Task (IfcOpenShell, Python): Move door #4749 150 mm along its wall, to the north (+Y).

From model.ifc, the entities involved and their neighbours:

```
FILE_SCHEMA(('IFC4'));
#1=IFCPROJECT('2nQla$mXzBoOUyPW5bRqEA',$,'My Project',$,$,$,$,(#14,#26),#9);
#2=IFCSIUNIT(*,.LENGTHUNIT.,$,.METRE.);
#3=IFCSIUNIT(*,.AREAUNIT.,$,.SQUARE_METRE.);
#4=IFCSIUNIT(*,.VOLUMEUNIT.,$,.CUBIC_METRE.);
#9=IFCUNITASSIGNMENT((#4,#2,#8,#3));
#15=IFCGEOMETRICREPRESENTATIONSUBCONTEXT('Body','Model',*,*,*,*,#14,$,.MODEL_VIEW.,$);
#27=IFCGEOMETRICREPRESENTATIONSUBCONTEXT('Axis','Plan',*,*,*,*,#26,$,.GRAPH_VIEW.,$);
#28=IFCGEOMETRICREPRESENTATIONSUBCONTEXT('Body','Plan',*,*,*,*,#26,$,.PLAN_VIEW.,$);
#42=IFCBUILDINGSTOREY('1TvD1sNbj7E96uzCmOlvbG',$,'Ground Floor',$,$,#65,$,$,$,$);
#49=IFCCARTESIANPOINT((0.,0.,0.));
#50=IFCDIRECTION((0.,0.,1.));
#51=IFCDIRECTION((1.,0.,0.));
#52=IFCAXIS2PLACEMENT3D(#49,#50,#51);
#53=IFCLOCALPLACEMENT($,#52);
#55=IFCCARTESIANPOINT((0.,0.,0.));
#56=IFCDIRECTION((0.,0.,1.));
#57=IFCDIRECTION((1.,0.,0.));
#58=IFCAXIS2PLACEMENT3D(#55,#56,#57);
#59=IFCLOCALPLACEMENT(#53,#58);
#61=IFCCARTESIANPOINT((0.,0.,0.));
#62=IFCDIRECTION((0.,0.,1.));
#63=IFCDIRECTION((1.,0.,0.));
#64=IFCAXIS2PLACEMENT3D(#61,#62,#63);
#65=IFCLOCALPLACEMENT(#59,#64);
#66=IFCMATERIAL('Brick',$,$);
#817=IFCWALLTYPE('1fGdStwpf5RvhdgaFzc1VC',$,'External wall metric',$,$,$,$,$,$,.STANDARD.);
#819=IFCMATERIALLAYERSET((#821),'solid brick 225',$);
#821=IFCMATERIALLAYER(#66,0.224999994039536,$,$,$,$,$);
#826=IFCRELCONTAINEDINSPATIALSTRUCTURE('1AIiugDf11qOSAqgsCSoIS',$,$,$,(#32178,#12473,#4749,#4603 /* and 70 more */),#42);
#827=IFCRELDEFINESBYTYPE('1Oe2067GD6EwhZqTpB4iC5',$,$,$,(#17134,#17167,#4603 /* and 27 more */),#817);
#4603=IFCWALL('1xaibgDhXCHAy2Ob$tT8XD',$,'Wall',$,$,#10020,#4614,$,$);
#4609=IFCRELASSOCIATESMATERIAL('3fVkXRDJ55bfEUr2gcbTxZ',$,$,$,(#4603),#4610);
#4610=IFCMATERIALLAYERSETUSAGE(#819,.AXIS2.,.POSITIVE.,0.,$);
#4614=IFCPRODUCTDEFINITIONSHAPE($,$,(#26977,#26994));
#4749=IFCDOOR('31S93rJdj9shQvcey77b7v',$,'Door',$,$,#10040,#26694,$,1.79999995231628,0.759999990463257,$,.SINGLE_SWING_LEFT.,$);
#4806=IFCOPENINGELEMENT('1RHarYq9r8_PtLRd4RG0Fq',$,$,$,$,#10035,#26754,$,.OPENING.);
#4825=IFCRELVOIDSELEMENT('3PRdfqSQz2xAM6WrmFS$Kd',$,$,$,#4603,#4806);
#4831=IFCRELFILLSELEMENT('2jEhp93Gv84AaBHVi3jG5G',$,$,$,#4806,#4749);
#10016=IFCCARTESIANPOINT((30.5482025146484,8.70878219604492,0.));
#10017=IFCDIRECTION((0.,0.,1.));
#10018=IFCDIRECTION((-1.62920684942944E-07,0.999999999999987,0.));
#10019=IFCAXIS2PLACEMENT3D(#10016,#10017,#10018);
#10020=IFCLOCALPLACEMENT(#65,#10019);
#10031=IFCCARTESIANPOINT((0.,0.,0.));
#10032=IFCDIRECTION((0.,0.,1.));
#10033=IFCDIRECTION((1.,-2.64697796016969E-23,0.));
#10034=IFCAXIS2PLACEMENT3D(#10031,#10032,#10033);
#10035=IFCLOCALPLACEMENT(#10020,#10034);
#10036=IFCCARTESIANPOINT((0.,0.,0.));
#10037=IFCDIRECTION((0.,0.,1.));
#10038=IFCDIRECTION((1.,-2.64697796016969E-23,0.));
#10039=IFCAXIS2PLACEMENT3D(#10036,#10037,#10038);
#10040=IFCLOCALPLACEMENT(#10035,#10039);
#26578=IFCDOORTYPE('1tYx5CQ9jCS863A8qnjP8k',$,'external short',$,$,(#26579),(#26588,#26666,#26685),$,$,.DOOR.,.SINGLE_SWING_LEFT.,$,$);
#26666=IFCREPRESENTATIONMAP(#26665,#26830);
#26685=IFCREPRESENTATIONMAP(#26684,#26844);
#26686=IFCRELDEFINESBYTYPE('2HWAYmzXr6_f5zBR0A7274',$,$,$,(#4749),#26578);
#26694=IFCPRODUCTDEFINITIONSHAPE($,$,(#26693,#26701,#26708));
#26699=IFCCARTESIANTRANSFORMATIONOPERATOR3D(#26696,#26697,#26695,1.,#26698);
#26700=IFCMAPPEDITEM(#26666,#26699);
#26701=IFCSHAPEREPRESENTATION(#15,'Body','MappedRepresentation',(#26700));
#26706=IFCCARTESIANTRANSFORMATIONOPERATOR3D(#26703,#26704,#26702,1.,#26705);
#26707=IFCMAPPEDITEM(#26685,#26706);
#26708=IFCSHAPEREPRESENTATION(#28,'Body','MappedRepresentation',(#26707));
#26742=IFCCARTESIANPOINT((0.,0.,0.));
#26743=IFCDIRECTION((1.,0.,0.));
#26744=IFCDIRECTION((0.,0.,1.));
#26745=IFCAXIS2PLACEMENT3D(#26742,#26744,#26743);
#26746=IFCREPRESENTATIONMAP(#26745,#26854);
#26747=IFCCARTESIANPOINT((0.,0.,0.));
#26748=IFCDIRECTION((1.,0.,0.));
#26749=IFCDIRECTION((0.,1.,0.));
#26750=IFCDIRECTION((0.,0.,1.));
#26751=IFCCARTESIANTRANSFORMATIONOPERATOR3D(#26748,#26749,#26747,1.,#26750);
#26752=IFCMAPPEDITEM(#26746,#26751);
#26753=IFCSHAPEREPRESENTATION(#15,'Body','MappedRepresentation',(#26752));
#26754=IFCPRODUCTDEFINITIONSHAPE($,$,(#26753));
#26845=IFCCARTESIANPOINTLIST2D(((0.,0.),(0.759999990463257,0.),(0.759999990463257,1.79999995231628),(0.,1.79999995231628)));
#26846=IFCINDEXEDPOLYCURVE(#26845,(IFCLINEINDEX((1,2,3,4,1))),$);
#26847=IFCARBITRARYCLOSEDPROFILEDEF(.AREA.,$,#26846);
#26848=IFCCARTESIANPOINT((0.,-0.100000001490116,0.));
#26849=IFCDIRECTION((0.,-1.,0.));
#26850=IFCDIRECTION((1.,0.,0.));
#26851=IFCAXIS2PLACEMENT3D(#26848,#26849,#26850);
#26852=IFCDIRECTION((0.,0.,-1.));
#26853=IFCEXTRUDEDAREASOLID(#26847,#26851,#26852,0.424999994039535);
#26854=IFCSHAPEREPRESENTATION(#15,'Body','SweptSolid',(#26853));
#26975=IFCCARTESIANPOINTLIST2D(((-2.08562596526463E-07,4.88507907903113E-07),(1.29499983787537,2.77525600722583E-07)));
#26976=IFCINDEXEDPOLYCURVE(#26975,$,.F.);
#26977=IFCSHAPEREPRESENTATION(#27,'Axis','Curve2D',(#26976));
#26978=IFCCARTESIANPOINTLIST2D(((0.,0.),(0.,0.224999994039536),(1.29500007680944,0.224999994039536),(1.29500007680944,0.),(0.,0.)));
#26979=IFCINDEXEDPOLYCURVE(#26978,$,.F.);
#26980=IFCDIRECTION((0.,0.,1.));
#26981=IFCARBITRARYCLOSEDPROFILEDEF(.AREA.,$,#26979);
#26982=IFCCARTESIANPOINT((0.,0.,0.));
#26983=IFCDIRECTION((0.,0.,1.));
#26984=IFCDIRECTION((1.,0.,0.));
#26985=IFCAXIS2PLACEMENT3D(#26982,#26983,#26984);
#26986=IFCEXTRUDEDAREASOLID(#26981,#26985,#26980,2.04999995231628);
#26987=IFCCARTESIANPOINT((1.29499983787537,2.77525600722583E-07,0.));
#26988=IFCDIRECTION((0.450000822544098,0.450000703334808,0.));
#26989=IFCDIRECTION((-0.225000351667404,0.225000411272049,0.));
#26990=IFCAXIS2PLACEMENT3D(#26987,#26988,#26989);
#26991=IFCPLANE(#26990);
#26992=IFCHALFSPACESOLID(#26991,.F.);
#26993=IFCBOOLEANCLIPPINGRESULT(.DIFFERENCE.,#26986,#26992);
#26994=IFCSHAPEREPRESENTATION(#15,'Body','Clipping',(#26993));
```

```python
import ifcopenshell
import ifcopenshell.api.geometry
import ifcopenshell.util.placement

model = ifcopenshell.open("model.ifc")

door = model.by_guid("31S93rJdj9shQvcey77b7v")
opening = door.FillsVoids[0].RelatingOpeningElement
wall = opening.VoidsElements[0].RelatingBuildingElement

wall_matrix = ifcopenshell.util.placement.get_local_placement(wall.ObjectPlacement)
shift = wall_matrix[:3, 0] * 0.15
before = ifcopenshell.util.placement.get_local_placement(door.ObjectPlacement)[:3, 3].copy()

# The door is placed relative to its opening, so it follows when the opening moves.
matrix = ifcopenshell.util.placement.get_local_placement(opening.ObjectPlacement)
matrix[:3, 3] += shift
ifcopenshell.api.geometry.edit_object_placement(
    model, product=opening, matrix=matrix, is_si=False, should_transform_children=True
)

after = ifcopenshell.util.placement.get_local_placement(door.ObjectPlacement)[:3, 3]
print("door moved by", (after - before).round(3) + 0.0)

model.write("model_updated.ifc")
```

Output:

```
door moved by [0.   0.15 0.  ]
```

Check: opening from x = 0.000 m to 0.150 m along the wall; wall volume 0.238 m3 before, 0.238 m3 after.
